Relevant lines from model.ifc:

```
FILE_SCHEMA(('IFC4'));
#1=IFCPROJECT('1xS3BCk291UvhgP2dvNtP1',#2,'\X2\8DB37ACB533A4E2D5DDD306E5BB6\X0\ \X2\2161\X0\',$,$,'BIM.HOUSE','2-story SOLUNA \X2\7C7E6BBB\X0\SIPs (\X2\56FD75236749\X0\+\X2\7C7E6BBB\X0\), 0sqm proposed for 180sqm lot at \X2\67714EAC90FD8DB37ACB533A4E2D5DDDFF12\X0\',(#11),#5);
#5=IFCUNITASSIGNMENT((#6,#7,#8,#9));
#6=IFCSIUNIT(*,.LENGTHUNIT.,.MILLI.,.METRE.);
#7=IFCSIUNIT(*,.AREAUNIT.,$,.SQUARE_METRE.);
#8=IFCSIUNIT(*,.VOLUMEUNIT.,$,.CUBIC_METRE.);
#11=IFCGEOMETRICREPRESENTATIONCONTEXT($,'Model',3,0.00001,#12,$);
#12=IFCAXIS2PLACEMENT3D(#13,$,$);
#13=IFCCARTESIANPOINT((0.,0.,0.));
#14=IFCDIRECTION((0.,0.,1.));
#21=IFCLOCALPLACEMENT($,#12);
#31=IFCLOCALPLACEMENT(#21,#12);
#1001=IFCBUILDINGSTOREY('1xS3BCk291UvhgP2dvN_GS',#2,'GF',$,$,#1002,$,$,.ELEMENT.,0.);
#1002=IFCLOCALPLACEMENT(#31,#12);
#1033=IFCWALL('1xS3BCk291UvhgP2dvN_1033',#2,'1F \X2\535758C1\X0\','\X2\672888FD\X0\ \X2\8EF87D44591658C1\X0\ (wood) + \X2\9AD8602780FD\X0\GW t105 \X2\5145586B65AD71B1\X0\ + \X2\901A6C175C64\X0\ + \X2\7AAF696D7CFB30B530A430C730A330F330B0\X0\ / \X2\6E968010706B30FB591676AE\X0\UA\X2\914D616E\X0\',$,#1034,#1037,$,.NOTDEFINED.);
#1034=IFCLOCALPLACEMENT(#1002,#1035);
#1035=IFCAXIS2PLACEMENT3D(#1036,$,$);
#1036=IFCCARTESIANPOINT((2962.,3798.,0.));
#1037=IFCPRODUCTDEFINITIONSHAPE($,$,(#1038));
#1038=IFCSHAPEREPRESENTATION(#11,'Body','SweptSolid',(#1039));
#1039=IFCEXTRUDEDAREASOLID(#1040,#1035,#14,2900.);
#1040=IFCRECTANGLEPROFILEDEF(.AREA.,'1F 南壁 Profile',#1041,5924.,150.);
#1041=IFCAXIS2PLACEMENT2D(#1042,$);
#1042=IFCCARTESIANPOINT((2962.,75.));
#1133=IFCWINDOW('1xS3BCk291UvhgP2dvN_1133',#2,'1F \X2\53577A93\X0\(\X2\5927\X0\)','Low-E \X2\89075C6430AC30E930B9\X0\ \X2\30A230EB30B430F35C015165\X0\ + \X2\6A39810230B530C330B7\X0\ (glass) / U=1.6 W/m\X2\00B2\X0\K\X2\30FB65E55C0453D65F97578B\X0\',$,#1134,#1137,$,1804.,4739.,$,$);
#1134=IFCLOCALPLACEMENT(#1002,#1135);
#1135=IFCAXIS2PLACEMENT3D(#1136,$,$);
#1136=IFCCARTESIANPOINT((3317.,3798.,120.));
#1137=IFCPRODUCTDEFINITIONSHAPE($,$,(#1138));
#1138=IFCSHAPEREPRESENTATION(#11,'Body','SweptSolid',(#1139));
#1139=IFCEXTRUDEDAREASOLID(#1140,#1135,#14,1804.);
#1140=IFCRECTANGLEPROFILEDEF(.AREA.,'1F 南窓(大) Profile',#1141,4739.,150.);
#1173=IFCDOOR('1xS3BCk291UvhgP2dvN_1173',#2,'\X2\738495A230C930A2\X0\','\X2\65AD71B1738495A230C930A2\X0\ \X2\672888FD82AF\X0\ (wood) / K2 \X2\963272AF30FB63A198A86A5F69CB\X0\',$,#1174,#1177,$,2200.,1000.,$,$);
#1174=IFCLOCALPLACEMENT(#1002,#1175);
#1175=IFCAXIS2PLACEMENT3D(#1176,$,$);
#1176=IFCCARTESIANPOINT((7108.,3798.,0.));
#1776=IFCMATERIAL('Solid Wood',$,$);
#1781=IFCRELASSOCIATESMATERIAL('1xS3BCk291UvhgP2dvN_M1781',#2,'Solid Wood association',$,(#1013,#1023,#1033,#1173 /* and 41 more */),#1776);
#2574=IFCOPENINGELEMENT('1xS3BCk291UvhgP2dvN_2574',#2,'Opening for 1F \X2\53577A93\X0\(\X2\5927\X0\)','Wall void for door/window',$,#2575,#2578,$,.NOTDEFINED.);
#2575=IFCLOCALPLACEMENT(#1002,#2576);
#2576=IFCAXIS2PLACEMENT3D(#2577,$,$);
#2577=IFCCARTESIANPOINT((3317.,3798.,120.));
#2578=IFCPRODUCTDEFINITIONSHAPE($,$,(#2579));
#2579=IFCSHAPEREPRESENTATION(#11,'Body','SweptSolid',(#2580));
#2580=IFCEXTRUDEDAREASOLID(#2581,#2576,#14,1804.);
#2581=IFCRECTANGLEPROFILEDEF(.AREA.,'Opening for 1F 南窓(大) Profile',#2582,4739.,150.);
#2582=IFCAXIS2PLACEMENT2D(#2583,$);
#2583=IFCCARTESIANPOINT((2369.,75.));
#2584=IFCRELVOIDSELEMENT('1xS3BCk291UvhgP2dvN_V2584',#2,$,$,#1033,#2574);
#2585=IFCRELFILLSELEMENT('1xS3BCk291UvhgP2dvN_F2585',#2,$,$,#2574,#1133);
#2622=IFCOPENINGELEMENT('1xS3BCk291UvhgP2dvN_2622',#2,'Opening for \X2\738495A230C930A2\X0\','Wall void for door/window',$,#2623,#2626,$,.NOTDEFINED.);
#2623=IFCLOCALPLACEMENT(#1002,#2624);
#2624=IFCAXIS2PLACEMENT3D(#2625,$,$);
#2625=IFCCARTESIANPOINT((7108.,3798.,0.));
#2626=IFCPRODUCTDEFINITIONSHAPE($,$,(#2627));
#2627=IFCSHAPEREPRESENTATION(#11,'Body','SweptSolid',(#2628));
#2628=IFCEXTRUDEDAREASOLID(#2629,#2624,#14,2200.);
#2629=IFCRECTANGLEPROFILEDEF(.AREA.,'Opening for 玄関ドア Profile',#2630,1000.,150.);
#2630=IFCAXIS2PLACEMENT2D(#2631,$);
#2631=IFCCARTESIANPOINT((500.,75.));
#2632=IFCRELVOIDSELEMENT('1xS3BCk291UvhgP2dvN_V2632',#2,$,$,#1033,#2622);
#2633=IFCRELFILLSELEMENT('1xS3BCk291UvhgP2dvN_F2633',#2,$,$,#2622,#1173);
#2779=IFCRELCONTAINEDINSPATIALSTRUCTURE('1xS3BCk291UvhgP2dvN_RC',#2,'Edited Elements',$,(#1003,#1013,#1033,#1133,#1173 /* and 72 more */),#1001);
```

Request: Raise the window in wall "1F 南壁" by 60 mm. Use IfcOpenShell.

```python
import numpy as np
import ifcopenshell
import ifcopenshell.api.geometry
import ifcopenshell.util.placement
import ifcopenshell.util.unit

model = ifcopenshell.open("model.ifc")
unit_scale = ifcopenshell.util.unit.calculate_unit_scale(model)

window = model.by_guid("1xS3BCk291UvhgP2dvN_1133")
opening = window.FillsVoids[0].RelatingOpeningElement
dz = 0.06 / unit_scale

shift = np.array([0.0, 0.0, dz])
# The window is not placed relative to its opening, so move both.
for product in (opening, window):
    matrix = ifcopenshell.util.placement.get_local_placement(product.ObjectPlacement)
    matrix[:3, 3] += shift
    ifcopenshell.api.geometry.edit_object_placement(model, product=product, matrix=matrix, is_si=False)

print(f"moved by {dz * unit_scale:+.3f} m")

model.write("model_edited.ifc")
```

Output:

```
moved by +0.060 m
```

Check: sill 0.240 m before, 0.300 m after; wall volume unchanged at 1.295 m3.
